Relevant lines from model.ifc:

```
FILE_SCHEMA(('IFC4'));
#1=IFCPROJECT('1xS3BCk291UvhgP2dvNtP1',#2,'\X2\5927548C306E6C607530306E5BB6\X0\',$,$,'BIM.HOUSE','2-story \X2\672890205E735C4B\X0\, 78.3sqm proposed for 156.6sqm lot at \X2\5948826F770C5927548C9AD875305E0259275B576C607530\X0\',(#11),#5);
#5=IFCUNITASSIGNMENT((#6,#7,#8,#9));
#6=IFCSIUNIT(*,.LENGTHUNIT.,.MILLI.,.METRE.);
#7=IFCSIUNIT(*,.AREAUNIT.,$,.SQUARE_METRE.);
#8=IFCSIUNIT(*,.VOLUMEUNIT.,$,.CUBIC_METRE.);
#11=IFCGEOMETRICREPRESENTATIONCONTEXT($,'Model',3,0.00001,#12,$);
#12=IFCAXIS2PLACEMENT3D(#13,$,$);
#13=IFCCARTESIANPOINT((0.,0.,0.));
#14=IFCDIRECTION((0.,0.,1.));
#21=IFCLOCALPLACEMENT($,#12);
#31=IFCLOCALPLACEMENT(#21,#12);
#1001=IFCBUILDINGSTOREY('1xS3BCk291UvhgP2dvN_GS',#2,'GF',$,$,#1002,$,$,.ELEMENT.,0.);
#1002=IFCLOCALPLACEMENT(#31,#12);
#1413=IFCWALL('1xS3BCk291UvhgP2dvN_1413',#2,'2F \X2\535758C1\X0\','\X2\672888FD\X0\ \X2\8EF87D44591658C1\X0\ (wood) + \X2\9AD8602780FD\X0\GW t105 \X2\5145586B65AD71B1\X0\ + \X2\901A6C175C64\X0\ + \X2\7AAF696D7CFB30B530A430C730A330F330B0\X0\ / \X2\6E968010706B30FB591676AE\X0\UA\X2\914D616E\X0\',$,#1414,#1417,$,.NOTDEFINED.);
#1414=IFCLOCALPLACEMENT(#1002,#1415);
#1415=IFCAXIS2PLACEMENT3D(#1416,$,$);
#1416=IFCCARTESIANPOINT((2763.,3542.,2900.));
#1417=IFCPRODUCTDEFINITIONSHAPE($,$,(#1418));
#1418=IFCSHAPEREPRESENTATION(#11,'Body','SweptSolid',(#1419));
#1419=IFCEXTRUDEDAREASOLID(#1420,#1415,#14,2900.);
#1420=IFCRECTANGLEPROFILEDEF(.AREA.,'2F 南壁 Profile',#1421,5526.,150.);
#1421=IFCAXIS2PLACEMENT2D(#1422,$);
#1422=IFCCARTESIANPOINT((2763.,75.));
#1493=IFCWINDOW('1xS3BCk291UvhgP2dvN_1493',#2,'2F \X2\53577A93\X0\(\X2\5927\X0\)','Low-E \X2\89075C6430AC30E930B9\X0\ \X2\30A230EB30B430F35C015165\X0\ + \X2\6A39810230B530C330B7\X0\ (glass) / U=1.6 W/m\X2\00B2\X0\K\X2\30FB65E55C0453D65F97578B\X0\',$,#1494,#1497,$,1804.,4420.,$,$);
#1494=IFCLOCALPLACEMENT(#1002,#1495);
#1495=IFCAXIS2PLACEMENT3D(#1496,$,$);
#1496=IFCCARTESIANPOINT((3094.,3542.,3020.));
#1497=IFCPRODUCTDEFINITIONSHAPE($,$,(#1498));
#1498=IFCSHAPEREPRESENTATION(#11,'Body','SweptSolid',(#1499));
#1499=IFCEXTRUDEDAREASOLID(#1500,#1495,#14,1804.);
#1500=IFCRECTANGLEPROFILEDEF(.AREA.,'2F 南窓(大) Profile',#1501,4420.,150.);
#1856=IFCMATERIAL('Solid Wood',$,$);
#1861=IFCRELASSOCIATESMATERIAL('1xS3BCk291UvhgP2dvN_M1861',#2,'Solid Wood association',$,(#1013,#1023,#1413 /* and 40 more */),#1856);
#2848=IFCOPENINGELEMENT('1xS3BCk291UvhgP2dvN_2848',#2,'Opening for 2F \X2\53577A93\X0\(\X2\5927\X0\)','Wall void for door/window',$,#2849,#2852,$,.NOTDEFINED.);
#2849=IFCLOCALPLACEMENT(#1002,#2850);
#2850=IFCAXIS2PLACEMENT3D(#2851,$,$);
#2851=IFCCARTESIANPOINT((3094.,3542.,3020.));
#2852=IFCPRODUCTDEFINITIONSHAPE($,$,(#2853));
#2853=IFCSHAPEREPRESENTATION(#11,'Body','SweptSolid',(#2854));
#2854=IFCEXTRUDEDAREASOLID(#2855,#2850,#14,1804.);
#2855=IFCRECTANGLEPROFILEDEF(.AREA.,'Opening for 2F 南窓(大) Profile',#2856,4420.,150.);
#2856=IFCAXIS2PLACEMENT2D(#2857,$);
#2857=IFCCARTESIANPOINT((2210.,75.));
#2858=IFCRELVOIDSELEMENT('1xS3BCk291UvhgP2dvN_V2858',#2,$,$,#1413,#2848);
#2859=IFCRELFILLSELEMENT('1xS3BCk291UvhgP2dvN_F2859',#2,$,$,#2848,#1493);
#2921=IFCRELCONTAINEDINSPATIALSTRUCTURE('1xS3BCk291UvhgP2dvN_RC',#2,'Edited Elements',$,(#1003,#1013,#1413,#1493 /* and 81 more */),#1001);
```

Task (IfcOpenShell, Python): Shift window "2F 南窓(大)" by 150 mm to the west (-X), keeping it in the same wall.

```python
import ifcopenshell
import ifcopenshell.api.geometry
import ifcopenshell.util.placement
import ifcopenshell.util.unit

model = ifcopenshell.open("model.ifc")
unit_scale = ifcopenshell.util.unit.calculate_unit_scale(model)

window = model.by_guid("1xS3BCk291UvhgP2dvN_1493")
opening = window.FillsVoids[0].RelatingOpeningElement
wall = opening.VoidsElements[0].RelatingBuildingElement

wall_matrix = ifcopenshell.util.placement.get_local_placement(wall.ObjectPlacement)
shift = wall_matrix[:3, 0] * -0.15 / unit_scale
before = ifcopenshell.util.placement.get_local_placement(window.ObjectPlacement)[:3, 3].copy()

# The window is not placed relative to its opening, so move both.
for product in (opening, window):
    matrix = ifcopenshell.util.placement.get_local_placement(product.ObjectPlacement)
    matrix[:3, 3] += shift
    ifcopenshell.api.geometry.edit_object_placement(model, product=product, matrix=matrix, is_si=False)

after = ifcopenshell.util.placement.get_local_placement(window.ObjectPlacement)[:3, 3]
print("window moved by", (after - before).round(3) + 0.0)

model.write("model_edited.ifc")
```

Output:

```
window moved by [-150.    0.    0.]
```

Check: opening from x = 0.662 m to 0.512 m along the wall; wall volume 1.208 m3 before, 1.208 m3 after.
